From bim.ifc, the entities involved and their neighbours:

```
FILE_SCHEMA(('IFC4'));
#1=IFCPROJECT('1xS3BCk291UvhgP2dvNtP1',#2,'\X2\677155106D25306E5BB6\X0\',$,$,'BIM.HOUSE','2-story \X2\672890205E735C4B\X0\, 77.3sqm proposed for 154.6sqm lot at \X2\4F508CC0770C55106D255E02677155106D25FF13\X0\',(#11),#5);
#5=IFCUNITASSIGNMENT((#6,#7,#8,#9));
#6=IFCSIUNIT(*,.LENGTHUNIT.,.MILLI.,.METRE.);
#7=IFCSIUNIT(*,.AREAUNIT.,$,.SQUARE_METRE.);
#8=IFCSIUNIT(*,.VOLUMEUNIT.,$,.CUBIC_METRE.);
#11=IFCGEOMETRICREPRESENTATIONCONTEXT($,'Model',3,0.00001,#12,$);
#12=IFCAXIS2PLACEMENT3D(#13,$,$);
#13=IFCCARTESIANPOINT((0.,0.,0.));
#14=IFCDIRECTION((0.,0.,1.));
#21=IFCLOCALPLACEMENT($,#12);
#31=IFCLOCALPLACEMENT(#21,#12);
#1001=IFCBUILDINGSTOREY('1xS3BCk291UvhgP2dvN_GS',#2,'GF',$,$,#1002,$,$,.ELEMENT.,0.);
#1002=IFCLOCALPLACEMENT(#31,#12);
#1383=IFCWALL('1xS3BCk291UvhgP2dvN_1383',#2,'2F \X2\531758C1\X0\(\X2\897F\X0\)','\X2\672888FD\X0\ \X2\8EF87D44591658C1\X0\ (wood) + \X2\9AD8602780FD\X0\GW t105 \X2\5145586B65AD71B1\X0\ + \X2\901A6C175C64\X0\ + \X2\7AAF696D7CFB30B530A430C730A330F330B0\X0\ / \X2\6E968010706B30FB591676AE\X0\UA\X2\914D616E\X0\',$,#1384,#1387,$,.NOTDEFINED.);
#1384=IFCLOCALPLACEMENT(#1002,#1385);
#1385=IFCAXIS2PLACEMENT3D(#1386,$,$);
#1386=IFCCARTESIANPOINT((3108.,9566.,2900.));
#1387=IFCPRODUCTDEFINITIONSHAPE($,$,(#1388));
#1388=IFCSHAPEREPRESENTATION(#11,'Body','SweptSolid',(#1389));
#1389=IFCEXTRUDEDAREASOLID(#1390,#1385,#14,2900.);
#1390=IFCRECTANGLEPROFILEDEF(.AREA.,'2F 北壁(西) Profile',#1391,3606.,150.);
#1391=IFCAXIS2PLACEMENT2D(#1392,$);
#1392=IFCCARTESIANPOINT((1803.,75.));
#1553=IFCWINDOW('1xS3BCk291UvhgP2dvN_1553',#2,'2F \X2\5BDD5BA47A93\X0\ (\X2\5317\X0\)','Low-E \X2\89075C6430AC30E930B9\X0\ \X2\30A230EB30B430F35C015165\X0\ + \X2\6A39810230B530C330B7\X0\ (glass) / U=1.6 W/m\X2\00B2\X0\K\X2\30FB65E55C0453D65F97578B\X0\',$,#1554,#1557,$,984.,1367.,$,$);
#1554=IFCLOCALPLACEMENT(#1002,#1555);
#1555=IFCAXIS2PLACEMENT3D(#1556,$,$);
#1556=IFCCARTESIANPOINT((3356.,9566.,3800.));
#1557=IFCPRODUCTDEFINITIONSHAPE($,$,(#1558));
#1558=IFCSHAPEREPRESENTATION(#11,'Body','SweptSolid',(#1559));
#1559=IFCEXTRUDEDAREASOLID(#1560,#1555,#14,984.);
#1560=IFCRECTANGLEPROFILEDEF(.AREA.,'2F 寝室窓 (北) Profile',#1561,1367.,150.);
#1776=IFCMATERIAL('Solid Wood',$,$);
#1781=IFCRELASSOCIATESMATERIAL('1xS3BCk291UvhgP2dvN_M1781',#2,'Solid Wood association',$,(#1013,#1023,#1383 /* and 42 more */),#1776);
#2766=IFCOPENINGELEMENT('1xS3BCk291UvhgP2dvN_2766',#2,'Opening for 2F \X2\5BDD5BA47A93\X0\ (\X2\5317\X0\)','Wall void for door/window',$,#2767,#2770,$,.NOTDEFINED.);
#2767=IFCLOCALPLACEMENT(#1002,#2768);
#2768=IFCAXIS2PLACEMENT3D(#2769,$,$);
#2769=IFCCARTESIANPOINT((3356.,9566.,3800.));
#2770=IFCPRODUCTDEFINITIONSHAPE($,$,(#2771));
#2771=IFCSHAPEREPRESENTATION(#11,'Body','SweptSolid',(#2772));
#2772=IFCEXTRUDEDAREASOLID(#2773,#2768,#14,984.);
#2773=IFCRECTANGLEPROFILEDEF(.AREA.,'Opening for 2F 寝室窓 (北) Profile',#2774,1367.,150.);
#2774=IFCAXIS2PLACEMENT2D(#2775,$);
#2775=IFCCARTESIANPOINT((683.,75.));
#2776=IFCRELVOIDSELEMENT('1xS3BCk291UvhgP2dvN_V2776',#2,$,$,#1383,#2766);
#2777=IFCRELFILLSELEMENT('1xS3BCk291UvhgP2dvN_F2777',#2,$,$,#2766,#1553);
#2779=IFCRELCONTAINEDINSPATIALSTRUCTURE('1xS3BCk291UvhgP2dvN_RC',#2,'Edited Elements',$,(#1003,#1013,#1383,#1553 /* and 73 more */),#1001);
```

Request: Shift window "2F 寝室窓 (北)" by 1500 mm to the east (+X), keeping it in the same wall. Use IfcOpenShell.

```python
import ifcopenshell
import ifcopenshell.api.geometry
import ifcopenshell.util.placement
import ifcopenshell.util.unit

model = ifcopenshell.open("bim.ifc")
unit_scale = ifcopenshell.util.unit.calculate_unit_scale(model)

window = model.by_guid("1xS3BCk291UvhgP2dvN_1553")
opening = window.FillsVoids[0].RelatingOpeningElement
wall = opening.VoidsElements[0].RelatingBuildingElement

wall_matrix = ifcopenshell.util.placement.get_local_placement(wall.ObjectPlacement)
shift = wall_matrix[:3, 0] * 1.5 / unit_scale
before = ifcopenshell.util.placement.get_local_placement(window.ObjectPlacement)[:3, 3].copy()

# The window is not placed relative to its opening, so move both.
for product in (opening, window):
    matrix = ifcopenshell.util.placement.get_local_placement(product.ObjectPlacement)
    matrix[:3, 3] += shift
    ifcopenshell.api.geometry.edit_object_placement(model, product=product, matrix=matrix, is_si=False)

after = ifcopenshell.util.placement.get_local_placement(window.ObjectPlacement)[:3, 3]
print("window moved by", (after - before).round(3) + 0.0)

model.write("bim-out.ifc")
```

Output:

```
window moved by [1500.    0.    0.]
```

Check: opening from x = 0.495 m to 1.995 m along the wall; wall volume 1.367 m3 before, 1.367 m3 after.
